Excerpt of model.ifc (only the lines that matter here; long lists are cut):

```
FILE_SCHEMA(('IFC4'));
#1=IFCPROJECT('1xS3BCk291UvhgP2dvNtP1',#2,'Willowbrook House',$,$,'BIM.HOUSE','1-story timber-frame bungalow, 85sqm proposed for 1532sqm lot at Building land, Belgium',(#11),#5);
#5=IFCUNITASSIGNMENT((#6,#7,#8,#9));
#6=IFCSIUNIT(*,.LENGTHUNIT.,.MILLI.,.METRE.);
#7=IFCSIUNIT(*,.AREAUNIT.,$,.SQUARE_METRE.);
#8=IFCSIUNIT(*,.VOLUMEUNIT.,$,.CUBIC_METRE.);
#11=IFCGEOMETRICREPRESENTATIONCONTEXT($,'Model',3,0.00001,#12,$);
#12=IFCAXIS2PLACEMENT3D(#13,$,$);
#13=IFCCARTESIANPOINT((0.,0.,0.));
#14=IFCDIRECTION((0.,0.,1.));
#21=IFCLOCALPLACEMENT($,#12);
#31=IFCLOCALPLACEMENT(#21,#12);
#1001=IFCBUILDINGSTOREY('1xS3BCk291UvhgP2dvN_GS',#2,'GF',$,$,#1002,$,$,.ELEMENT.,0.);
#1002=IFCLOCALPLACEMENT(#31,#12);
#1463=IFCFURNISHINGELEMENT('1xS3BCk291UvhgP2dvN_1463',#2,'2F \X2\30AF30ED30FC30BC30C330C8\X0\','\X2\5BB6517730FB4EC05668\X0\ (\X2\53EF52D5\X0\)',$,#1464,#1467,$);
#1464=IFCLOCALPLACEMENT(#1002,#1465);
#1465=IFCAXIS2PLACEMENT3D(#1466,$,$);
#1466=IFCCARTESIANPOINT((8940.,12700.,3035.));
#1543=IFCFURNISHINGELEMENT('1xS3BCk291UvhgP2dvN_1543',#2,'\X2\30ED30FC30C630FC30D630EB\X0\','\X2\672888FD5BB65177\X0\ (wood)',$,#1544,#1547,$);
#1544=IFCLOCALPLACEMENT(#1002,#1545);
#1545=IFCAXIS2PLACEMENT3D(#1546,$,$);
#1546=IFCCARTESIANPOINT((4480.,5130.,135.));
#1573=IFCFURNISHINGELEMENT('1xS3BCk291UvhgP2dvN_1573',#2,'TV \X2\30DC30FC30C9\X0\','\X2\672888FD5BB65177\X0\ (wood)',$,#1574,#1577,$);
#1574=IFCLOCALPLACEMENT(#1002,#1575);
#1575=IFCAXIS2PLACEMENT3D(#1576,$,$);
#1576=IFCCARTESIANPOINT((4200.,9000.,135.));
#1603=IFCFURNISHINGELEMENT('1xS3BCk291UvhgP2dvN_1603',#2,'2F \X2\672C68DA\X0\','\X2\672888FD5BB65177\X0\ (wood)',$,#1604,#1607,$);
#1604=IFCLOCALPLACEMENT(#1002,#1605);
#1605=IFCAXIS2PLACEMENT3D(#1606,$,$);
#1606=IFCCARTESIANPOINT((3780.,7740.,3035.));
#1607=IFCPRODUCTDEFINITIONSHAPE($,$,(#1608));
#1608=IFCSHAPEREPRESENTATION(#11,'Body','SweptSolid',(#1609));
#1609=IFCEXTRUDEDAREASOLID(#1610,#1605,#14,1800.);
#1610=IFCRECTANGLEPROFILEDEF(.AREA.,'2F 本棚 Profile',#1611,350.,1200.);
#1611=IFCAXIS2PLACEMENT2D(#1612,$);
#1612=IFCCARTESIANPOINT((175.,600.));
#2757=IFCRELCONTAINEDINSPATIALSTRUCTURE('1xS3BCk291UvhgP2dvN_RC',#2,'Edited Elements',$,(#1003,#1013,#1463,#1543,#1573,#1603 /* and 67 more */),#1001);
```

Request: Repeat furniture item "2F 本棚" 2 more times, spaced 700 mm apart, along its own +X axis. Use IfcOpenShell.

```python
import ifcopenshell
import ifcopenshell.api.geometry
import ifcopenshell.api.root
import ifcopenshell.util.element
import ifcopenshell.util.placement
import ifcopenshell.util.unit

model = ifcopenshell.open("model.ifc")
unit_scale = ifcopenshell.util.unit.calculate_unit_scale(model)


def reuse_history(source, copy):
    """copy_class also copies each property set's owner history, people and application; keep the originals."""
    for rel in copy.IsDefinedBy:
        if rel.is_a("IfcRelDefinesByProperties") and (history := rel.RelatingPropertyDefinition.OwnerHistory):
            rel.RelatingPropertyDefinition.OwnerHistory = source.OwnerHistory
            ifcopenshell.util.element.remove_deep2(model, history)


source = model.by_guid("1xS3BCk291UvhgP2dvN_1603")
base = ifcopenshell.util.placement.get_local_placement(source.ObjectPlacement)
step = base[:3, 0] * 0.7 / unit_scale

for i in range(1, 3):
    copy = ifcopenshell.api.root.copy_class(model, product=source)
    copy.Representation = ifcopenshell.util.element.copy_deep(
        model, source.Representation, exclude=["IfcGeometricRepresentationContext", "IfcRepresentationMap"]
    )
    reuse_history(source, copy)
    matrix = base.copy()
    matrix[:3, 3] += i * step
    print("added at", matrix[:3, 3].round(3) + 0.0)
    ifcopenshell.api.geometry.edit_object_placement(model, product=copy, matrix=matrix, is_si=False)

model.write("model-out.ifc")
```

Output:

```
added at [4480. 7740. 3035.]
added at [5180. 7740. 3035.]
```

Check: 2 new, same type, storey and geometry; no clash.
